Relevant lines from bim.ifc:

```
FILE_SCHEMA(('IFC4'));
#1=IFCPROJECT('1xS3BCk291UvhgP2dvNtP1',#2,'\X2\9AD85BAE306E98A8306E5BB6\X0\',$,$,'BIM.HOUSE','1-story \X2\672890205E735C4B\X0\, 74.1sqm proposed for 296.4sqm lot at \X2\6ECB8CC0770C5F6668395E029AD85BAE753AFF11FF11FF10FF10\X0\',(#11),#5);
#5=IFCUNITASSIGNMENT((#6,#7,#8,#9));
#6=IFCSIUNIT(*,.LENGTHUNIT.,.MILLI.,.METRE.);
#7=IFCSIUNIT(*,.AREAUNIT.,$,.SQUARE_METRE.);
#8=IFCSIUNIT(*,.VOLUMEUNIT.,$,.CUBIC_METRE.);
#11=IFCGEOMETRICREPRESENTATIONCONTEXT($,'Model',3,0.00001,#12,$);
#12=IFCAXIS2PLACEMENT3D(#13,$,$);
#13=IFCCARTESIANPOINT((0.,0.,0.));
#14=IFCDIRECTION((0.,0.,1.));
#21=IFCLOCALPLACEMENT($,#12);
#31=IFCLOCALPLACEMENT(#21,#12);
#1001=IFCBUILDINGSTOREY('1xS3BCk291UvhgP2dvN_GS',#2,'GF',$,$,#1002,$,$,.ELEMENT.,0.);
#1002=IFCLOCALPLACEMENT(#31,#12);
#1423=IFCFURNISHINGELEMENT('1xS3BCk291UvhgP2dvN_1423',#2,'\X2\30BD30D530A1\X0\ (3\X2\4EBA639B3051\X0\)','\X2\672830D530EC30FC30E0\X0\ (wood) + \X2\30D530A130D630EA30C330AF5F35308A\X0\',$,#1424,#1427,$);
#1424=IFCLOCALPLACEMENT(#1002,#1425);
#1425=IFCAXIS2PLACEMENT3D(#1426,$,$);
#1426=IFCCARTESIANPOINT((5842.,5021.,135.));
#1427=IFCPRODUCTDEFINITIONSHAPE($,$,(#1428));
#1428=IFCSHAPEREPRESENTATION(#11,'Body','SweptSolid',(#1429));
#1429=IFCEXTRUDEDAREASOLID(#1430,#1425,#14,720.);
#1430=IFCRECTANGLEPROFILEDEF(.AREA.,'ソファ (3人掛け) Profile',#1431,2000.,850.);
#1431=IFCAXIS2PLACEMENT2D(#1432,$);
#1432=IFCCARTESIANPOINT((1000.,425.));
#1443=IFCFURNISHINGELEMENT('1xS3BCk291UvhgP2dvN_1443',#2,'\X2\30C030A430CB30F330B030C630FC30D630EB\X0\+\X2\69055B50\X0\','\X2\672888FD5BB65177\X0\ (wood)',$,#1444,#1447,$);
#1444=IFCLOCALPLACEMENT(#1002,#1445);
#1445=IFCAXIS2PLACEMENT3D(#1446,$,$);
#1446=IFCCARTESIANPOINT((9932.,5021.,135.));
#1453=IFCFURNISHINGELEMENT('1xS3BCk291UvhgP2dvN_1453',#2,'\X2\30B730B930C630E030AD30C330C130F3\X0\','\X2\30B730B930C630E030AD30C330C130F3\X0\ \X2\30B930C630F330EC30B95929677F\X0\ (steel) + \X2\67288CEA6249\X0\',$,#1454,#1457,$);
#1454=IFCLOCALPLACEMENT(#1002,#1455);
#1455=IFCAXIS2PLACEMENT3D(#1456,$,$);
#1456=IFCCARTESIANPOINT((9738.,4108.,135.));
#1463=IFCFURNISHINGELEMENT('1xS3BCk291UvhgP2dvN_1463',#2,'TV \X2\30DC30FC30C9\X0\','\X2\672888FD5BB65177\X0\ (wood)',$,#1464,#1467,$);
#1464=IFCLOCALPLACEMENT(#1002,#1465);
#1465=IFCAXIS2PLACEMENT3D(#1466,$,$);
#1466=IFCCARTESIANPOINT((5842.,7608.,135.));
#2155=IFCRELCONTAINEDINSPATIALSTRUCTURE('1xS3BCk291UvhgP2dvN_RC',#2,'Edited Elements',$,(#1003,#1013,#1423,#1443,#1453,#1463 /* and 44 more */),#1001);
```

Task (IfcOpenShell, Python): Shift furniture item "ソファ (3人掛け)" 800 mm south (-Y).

```python
import ifcopenshell
import ifcopenshell.api.geometry
import ifcopenshell.util.placement
import ifcopenshell.util.unit

model = ifcopenshell.open("bim.ifc")
unit_scale = ifcopenshell.util.unit.calculate_unit_scale(model)

item = model.by_id(1423)
matrix = ifcopenshell.util.placement.get_local_placement(item.ObjectPlacement)
matrix[1, 3] -= 0.8 / unit_scale
ifcopenshell.api.geometry.edit_object_placement(model, product=item, matrix=matrix, is_si=False)

print(ifcopenshell.util.placement.get_local_placement(item.ObjectPlacement).round(3) + 0.0)

model.write("bim_v2.ifc")
```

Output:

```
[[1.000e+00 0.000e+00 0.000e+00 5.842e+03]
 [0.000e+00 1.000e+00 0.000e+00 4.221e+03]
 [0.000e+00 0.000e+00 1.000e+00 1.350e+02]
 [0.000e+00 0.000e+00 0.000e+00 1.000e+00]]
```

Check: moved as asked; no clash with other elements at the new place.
